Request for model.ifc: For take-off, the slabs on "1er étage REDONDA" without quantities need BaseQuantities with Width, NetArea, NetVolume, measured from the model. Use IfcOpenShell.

First a look at what the model holds.

```python
import ifcopenshell
import ifcopenshell.util.element
import ifcopenshell.util.unit

model = ifcopenshell.open("model.ifc")
print(model.schema)
for unit_type in ("LENGTHUNIT", "AREAUNIT", "VOLUMEUNIT"):
    print(unit_type, ifcopenshell.util.unit.calculate_unit_scale(model, unit_type))
storey = next(s for s in model.by_type("IfcBuildingStorey") if s.Name == "1er étage REDONDA")
slabs = [e for e in ifcopenshell.util.element.get_decomposition(storey) if e.is_a("IfcSlab")]
for e in sorted(slabs, key=lambda e: e.id()):
    print(e.id(), e.is_a(), e.Name, list(ifcopenshell.util.element.get_psets(e, qtos_only=True)), sep=" | ")
```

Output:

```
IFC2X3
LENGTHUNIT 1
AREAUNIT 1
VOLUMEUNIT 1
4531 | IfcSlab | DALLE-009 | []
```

```python
import ifcopenshell
import ifcopenshell.api.pset
import ifcopenshell.geom
import ifcopenshell.util.element
import ifcopenshell.util.shape
import ifcopenshell.util.unit

model = ifcopenshell.open("model.ifc")
unit_scale = ifcopenshell.util.unit.calculate_unit_scale(model)
area_scale = ifcopenshell.util.unit.calculate_unit_scale(model, "AREAUNIT")
volume_scale = ifcopenshell.util.unit.calculate_unit_scale(model, "VOLUMEUNIT")
settings = ifcopenshell.geom.settings()

storey = next(s for s in model.by_type("IfcBuildingStorey") if s.Name == "1er étage REDONDA")
slabs = [e for e in ifcopenshell.util.element.get_decomposition(storey) if e.is_a("IfcSlab")]

for e in sorted(slabs, key=lambda e: e.id()):
    if ifcopenshell.util.element.get_psets(e, qtos_only=True, should_inherit=False):
        continue
    # Geometry comes back in metres, in the element's own axes.
    shape = ifcopenshell.geom.create_shape(settings, e)
    values = {
        "Width": ifcopenshell.util.shape.get_z(shape.geometry) / unit_scale,
        "NetArea": ifcopenshell.util.shape.get_footprint_area(shape.geometry) / area_scale,
        "NetVolume": ifcopenshell.util.shape.get_volume(shape.geometry) / volume_scale,
    }
    qto = ifcopenshell.api.pset.add_qto(model, product=e, name="BaseQuantities")
    ifcopenshell.api.pset.edit_qto(model, qto=qto, properties=values)
    print(e.id(), {k: round(v, 3) for k, v in values.items()})

model.write("model-out.ifc")
```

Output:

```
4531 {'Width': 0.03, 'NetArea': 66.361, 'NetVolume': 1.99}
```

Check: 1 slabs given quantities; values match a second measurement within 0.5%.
